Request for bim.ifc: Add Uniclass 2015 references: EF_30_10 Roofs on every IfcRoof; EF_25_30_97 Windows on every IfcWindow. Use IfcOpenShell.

First a look at what the model holds.

```python
import ifcopenshell

model = ifcopenshell.open("bim.ifc")
print(model.schema)
print("classifications:", [c.Name for c in model.by_type("IfcClassification")])
for ifc_class in ("IfcDoor", "IfcRoof", "IfcStair", "IfcWall", "IfcWindow"):
    print(ifc_class, len(model.by_type(ifc_class)))
```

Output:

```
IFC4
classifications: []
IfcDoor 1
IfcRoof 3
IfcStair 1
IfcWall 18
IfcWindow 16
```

```python
import ifcopenshell
import ifcopenshell.api.classification

model = ifcopenshell.open("bim.ifc")

system = ifcopenshell.api.classification.add_classification(model, classification="Uniclass 2015")

codes = {
    "IfcRoof": ("EF_30_10", "Roofs"),
    "IfcWindow": ("EF_25_30_97", "Windows"),
}
for ifc_class, (code, name) in codes.items():
    products = model.by_type(ifc_class)
    ifcopenshell.api.classification.add_reference(
        model, products=products, classification=system, identification=code, name=name
    )
    print(code, len(products))

model.write("bim_updated.ifc")
```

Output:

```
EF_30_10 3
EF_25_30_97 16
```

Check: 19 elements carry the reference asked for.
